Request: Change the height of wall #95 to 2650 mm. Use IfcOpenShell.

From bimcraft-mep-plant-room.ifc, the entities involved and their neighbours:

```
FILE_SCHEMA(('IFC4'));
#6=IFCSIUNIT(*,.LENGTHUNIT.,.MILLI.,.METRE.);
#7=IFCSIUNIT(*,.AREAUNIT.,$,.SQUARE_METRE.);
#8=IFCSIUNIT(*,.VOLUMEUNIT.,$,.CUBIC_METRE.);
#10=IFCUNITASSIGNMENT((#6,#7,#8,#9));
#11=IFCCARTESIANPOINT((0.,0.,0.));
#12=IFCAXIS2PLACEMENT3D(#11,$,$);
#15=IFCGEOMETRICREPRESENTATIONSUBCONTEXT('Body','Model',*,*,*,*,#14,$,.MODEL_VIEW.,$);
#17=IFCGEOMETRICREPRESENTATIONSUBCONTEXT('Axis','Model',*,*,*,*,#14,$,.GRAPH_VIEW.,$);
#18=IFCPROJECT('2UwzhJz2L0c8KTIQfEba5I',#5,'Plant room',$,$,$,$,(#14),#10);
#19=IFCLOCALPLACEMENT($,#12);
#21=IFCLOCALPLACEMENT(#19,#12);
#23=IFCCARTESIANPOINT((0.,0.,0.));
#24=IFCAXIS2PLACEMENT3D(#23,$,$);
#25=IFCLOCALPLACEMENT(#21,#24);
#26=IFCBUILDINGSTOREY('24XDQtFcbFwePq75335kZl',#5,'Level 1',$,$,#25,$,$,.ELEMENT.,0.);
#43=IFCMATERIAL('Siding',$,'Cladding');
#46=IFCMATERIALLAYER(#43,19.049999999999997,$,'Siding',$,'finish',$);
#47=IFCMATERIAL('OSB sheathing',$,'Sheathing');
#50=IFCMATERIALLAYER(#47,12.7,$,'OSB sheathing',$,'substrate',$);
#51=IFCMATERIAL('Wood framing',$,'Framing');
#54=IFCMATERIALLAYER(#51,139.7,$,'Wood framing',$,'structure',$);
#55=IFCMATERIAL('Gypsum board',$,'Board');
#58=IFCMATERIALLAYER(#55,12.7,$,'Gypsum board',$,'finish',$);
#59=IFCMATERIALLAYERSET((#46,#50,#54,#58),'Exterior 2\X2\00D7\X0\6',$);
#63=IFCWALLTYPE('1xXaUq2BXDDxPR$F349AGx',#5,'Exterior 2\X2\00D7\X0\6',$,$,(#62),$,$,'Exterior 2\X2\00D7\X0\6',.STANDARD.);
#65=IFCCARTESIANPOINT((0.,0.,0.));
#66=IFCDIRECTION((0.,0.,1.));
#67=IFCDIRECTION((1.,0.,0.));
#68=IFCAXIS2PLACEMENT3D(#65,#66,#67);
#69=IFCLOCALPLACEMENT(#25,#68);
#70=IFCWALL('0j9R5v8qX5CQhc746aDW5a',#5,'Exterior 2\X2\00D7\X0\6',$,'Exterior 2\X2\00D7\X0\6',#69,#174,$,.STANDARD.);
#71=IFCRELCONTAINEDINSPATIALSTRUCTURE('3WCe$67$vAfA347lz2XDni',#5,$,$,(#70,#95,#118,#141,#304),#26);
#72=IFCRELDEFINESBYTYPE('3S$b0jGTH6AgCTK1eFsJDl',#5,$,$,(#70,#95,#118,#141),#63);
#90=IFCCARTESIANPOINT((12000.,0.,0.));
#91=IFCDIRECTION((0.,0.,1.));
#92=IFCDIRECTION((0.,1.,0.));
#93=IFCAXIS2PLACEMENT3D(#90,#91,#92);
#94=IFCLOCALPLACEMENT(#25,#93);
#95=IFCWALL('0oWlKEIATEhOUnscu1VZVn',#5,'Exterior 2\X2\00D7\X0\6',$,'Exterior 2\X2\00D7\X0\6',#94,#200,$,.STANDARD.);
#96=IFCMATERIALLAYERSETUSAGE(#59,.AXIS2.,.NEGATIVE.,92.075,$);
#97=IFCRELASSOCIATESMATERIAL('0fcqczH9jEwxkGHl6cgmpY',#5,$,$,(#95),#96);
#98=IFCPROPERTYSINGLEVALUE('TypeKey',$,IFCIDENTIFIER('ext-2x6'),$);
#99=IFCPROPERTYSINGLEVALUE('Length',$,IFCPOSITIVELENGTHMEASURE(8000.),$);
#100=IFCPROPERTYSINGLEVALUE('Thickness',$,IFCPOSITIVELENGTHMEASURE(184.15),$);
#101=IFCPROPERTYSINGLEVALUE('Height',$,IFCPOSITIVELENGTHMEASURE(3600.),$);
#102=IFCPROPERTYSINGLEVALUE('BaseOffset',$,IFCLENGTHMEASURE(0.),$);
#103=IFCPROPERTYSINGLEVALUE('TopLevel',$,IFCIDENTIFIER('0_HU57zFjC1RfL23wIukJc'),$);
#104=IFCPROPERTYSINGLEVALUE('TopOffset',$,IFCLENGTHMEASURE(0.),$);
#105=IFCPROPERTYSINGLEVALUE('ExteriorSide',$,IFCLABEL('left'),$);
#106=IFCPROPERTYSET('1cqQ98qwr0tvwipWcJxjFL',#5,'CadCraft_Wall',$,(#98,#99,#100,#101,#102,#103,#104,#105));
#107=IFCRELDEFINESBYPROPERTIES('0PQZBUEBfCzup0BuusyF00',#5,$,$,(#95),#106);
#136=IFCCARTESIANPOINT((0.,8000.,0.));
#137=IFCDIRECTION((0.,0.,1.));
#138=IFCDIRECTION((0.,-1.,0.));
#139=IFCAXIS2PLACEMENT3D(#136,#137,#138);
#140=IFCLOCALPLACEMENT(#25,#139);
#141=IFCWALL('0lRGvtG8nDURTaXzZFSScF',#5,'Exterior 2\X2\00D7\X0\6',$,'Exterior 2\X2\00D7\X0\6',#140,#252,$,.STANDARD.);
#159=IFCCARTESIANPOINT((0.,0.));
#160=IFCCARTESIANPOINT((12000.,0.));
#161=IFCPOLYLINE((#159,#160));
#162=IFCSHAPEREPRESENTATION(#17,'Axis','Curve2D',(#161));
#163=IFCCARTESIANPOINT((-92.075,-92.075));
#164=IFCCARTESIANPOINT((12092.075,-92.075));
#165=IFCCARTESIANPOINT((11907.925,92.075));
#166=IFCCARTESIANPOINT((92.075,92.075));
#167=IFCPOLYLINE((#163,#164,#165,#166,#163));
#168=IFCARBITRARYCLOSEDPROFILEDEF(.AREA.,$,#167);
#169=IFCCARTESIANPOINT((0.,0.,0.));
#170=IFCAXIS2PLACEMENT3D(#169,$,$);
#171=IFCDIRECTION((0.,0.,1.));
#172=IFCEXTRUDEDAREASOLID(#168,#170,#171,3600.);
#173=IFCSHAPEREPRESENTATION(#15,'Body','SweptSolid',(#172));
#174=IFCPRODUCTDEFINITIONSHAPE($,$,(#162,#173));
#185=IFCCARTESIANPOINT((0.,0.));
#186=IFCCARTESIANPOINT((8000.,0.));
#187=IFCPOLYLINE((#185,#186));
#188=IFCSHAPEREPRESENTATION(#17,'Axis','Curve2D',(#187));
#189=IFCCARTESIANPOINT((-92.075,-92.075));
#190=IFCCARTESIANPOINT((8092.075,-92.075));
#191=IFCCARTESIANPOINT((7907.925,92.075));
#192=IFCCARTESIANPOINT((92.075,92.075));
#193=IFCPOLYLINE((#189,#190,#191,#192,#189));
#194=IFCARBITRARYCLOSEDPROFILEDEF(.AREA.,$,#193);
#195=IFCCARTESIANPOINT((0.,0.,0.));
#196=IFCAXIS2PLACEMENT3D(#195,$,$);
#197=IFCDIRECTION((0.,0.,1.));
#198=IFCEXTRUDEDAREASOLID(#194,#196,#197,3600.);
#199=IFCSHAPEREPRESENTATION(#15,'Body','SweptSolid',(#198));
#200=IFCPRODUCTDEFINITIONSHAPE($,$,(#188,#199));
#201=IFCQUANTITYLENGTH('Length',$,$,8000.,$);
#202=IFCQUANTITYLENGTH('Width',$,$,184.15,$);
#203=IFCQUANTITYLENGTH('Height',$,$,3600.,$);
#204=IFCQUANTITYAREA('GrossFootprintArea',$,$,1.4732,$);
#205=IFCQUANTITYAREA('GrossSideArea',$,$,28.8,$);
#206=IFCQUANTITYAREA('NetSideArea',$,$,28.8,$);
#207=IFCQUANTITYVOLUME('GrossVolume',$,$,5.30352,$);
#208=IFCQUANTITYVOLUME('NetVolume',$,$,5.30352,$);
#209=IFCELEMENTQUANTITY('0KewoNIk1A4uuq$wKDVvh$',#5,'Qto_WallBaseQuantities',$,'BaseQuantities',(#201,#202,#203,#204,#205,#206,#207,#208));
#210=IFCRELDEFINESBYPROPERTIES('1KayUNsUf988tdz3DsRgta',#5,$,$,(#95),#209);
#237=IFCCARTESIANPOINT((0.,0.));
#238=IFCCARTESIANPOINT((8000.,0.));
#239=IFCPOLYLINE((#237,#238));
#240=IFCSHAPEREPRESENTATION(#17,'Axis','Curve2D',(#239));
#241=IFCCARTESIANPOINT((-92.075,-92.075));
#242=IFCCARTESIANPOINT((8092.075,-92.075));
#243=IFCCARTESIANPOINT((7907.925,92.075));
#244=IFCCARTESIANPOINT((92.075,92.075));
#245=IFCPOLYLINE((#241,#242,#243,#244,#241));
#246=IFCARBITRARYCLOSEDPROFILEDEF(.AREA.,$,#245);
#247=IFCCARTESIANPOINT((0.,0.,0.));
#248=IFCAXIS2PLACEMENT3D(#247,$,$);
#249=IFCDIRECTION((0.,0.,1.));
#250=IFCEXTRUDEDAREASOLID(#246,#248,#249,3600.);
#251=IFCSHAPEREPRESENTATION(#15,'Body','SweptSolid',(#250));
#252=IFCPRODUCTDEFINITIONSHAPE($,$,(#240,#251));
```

```python
import ifcopenshell
import ifcopenshell.api.pset
import ifcopenshell.geom
import ifcopenshell.util.element
import ifcopenshell.util.representation
import ifcopenshell.util.shape
import ifcopenshell.util.unit

model = ifcopenshell.open("bimcraft-mep-plant-room.ifc")
unit_scale = ifcopenshell.util.unit.calculate_unit_scale(model)
area_scale = ifcopenshell.util.unit.calculate_unit_scale(model, "AREAUNIT")
volume_scale = ifcopenshell.util.unit.calculate_unit_scale(model, "VOLUMEUNIT")
settings = ifcopenshell.geom.settings()


def volume(element):
    """Net volume in cubic metres, openings subtracted."""
    shape = ifcopenshell.geom.create_shape(settings, element)
    return ifcopenshell.util.shape.get_volume(shape.geometry)


wall = model.by_guid("0oWlKEIATEhOUnscu1VZVn")
before = volume(wall)

body = ifcopenshell.util.representation.get_representation(wall, "Model", "Body")
solid = body.Items[0]
old_height = solid.Depth
solid.Depth = 2650.0
after = volume(wall)
thickness = 0.1841  # wall thickness in metres

# Update the stored height, areas and volumes.
pset = model.by_id(ifcopenshell.util.element.get_pset(wall, "CadCraft_Wall", should_inherit=False)["id"])
ifcopenshell.api.pset.edit_pset(model, pset=pset, properties={
    "Height": model.create_entity("IfcPositiveLengthMeasure", solid.Depth),
})
qto = model.by_id(ifcopenshell.util.element.get_pset(wall, "Qto_WallBaseQuantities", should_inherit=False)["id"])
ifcopenshell.api.pset.edit_qto(model, qto=qto, properties={
    "Height": solid.Depth,
    "GrossSideArea": ifcopenshell.util.element.get_pset(wall, "Qto_WallBaseQuantities", "GrossSideArea") * solid.Depth / old_height,
    "NetSideArea": after / thickness / area_scale,
    "GrossVolume": ifcopenshell.util.element.get_pset(wall, "Qto_WallBaseQuantities", "GrossVolume") * solid.Depth / old_height,
    "NetVolume": after / volume_scale,
})

print(f"height {old_height:g} -> {solid.Depth:g}, volume {before:.3f} -> {after:.3f} m3")

model.write("bimcraft-mep-plant-room_edited.ifc")
```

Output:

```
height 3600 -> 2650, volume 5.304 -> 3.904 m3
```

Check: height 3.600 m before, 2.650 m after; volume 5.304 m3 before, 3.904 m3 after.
